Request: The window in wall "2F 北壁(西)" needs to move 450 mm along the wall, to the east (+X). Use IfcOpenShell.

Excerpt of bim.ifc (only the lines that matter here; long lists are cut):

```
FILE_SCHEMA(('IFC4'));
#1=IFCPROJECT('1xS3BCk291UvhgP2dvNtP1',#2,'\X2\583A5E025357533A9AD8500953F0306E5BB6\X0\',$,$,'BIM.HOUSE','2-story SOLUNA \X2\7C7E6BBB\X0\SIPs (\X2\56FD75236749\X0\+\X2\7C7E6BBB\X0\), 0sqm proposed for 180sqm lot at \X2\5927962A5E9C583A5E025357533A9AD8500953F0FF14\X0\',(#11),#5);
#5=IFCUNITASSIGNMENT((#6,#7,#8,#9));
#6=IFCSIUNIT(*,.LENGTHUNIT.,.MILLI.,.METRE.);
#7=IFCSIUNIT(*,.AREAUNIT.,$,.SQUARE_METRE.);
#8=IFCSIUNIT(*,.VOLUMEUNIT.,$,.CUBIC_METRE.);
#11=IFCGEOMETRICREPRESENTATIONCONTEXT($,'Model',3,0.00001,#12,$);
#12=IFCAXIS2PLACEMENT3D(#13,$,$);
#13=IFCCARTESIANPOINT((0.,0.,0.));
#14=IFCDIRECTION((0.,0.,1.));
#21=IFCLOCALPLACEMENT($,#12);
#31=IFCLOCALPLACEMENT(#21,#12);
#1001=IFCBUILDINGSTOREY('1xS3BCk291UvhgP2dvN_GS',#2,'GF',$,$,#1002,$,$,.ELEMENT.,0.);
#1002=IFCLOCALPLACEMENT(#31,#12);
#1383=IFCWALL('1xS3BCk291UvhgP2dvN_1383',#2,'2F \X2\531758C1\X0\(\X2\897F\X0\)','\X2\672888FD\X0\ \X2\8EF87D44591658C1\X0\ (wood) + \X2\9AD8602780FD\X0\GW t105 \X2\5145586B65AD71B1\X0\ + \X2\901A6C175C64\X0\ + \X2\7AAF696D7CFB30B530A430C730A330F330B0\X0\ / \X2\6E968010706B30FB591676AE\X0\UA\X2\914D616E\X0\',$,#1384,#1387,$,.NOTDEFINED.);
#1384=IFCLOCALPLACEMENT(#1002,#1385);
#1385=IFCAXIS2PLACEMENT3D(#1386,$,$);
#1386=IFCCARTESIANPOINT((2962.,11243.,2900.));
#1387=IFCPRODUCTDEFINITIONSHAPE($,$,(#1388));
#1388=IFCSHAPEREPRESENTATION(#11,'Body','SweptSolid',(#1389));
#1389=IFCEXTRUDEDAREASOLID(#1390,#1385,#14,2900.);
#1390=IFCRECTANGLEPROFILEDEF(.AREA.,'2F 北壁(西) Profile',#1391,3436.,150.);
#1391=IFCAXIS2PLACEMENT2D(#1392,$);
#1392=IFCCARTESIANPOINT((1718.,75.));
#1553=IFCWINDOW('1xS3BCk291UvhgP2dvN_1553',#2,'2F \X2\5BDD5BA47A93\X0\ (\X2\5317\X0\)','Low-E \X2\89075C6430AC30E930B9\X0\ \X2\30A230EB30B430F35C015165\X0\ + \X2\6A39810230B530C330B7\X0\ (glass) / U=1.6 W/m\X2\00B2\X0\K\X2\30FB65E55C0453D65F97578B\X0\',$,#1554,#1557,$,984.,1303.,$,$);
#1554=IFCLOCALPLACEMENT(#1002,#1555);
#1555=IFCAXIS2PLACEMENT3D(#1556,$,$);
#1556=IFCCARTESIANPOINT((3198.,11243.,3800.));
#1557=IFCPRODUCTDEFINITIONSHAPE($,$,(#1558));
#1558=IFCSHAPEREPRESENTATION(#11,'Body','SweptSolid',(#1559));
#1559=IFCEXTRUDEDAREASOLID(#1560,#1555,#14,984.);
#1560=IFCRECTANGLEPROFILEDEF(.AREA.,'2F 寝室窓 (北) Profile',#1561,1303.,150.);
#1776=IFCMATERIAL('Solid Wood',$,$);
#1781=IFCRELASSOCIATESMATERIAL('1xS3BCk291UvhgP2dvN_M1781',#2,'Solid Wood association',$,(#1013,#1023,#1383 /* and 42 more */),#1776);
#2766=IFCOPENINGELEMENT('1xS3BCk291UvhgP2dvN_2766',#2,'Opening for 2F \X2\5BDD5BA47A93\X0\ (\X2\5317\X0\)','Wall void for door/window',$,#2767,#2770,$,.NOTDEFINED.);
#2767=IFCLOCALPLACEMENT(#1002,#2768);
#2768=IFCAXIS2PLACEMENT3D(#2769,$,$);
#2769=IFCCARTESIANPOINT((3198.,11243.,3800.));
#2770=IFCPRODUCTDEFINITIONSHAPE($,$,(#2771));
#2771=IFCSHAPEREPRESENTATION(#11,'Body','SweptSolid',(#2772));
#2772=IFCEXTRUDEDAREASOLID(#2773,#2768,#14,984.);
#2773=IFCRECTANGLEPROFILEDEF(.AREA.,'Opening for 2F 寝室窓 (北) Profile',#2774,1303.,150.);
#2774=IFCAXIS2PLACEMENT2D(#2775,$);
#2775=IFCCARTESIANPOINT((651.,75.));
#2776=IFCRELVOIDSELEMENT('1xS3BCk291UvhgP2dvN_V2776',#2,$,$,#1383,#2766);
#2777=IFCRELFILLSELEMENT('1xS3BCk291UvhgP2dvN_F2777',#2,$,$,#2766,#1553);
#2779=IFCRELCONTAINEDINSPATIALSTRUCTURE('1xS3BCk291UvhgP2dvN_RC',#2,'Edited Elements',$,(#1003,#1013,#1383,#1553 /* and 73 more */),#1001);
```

```python
import ifcopenshell
import ifcopenshell.api.geometry
import ifcopenshell.util.placement

model = ifcopenshell.open("bim.ifc")

window = model.by_guid("1xS3BCk291UvhgP2dvN_1553")
opening = window.FillsVoids[0].RelatingOpeningElement
wall = opening.VoidsElements[0].RelatingBuildingElement

wall_matrix = ifcopenshell.util.placement.get_local_placement(wall.ObjectPlacement)
shift = wall_matrix[:3, 0] * 450.0
before = ifcopenshell.util.placement.get_local_placement(window.ObjectPlacement)[:3, 3].copy()

# The window is not placed relative to its opening, so move both.
for product in (opening, window):
    matrix = ifcopenshell.util.placement.get_local_placement(product.ObjectPlacement)
    matrix[:3, 3] += shift
    ifcopenshell.api.geometry.edit_object_placement(model, product=product, matrix=matrix, is_si=False)

after = ifcopenshell.util.placement.get_local_placement(window.ObjectPlacement)[:3, 3]
print("window moved by", (after - before).round(3) + 0.0)

model.write("bim_rev.ifc")
```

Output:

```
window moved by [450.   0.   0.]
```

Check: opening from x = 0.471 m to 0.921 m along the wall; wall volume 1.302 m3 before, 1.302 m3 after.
